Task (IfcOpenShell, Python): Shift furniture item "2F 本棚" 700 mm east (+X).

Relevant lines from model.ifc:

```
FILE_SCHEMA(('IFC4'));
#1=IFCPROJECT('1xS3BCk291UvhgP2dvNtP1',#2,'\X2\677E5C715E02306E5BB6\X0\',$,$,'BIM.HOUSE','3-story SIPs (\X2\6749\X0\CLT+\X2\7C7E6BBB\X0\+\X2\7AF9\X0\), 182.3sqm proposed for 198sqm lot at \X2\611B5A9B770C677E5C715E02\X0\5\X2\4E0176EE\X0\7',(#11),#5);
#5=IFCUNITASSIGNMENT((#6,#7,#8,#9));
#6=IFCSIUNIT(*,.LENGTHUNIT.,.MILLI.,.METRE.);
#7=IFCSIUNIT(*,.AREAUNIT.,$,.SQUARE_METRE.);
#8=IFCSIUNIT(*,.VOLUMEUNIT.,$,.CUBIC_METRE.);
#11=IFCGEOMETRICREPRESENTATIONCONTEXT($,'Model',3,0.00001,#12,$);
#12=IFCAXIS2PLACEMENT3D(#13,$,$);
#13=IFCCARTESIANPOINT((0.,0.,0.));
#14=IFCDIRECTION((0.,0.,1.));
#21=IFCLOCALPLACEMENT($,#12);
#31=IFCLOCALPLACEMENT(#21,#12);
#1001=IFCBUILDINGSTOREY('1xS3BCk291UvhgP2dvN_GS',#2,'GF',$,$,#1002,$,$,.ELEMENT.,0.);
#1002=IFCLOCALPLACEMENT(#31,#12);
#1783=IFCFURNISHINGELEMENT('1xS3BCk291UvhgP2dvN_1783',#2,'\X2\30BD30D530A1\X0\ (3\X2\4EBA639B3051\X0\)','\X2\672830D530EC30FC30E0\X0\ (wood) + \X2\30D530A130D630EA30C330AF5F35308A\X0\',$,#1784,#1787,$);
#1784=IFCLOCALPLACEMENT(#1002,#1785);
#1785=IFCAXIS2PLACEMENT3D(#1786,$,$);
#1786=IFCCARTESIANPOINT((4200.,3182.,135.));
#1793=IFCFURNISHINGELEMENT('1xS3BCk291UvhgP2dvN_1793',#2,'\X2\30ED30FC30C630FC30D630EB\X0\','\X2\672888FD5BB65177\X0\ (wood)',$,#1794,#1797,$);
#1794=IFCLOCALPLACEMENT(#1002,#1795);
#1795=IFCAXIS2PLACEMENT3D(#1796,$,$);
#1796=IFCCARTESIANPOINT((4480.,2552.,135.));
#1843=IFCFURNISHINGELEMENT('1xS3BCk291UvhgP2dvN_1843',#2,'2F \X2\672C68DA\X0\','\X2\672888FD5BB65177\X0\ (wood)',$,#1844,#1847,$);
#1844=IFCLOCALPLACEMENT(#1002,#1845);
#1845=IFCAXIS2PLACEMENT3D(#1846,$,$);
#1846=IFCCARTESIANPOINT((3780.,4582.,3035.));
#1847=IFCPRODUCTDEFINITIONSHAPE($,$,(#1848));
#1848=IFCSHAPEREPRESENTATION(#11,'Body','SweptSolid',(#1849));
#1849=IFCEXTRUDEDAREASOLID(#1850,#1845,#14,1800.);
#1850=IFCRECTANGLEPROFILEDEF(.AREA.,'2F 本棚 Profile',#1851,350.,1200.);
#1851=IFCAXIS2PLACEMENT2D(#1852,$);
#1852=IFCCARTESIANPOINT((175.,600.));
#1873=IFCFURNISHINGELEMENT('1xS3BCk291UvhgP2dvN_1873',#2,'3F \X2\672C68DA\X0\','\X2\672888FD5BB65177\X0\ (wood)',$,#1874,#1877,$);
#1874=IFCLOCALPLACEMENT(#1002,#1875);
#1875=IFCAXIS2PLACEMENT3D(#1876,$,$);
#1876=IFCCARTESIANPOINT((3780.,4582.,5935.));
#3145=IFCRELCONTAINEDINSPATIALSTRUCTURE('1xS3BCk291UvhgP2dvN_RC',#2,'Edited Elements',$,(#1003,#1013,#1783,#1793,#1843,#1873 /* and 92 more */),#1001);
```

```python
import ifcopenshell
import ifcopenshell.api.geometry
import ifcopenshell.util.placement
import ifcopenshell.util.unit

model = ifcopenshell.open("model.ifc")
unit_scale = ifcopenshell.util.unit.calculate_unit_scale(model)

item = model.by_guid("1xS3BCk291UvhgP2dvN_1843")
matrix = ifcopenshell.util.placement.get_local_placement(item.ObjectPlacement)
matrix[0, 3] += 0.7 / unit_scale
ifcopenshell.api.geometry.edit_object_placement(model, product=item, matrix=matrix, is_si=False)

print(ifcopenshell.util.placement.get_local_placement(item.ObjectPlacement).round(3) + 0.0)

model.write("model_edited.ifc")
```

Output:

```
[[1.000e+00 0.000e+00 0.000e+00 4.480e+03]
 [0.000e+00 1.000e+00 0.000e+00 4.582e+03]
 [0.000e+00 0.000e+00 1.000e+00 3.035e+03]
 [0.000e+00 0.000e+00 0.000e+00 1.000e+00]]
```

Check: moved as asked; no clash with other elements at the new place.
